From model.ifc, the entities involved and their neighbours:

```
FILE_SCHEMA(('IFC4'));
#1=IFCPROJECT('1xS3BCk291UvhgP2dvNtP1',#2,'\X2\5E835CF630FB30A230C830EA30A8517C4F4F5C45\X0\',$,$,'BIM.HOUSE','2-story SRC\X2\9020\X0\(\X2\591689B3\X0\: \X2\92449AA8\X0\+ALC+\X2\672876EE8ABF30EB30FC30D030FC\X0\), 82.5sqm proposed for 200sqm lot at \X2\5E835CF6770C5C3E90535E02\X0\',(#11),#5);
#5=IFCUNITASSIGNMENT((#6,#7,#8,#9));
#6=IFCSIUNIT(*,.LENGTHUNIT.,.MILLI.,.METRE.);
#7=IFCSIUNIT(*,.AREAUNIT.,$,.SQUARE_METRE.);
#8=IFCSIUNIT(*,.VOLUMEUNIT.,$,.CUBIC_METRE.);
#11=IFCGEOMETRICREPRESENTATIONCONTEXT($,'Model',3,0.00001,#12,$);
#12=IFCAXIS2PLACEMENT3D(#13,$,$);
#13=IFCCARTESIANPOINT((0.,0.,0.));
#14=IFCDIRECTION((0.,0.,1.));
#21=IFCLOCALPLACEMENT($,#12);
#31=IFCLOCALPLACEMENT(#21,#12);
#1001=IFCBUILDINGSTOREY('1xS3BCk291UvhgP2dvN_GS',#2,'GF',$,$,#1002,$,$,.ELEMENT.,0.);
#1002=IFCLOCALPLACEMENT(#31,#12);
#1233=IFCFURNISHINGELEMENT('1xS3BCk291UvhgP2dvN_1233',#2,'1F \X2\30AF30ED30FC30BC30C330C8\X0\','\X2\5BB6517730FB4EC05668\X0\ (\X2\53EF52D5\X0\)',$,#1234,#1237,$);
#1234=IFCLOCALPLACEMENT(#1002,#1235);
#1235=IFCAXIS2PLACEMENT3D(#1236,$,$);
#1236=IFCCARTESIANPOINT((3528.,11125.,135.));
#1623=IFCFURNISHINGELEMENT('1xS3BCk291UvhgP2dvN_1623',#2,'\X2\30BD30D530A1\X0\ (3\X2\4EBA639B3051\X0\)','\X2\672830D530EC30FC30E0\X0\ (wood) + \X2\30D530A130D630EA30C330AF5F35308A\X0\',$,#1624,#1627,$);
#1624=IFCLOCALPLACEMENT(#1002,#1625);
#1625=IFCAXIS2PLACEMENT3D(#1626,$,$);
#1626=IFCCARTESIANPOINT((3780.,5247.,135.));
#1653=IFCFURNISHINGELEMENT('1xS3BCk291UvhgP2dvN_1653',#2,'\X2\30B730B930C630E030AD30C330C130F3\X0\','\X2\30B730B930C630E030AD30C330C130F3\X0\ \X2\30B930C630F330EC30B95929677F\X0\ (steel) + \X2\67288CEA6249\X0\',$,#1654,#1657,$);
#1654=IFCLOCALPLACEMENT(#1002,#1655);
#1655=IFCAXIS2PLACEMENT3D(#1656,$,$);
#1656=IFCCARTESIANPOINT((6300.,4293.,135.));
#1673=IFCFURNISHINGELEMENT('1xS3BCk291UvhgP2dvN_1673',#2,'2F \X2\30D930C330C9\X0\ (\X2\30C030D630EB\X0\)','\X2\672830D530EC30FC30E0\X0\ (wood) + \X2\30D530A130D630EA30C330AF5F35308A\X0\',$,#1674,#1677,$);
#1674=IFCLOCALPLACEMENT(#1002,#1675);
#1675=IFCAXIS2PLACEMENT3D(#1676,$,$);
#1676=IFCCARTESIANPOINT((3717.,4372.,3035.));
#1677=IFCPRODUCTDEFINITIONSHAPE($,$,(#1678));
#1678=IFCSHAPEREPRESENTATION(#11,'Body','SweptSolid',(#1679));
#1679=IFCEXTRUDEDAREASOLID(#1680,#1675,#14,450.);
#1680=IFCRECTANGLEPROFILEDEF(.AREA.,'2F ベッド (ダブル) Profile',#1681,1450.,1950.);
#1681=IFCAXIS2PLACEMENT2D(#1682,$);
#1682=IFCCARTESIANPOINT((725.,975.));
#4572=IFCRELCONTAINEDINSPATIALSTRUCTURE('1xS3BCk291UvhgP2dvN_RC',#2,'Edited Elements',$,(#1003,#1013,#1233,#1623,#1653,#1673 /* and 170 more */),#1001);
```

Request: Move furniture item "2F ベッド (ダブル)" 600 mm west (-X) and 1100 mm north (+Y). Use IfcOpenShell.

```python
import ifcopenshell
import ifcopenshell.api.geometry
import ifcopenshell.util.placement

model = ifcopenshell.open("model.ifc")

item = model.by_id(1673)
matrix = ifcopenshell.util.placement.get_local_placement(item.ObjectPlacement)
matrix[0, 3] -= 600.0
matrix[1, 3] += 1100.0
ifcopenshell.api.geometry.edit_object_placement(model, product=item, matrix=matrix, is_si=False)

print(ifcopenshell.util.placement.get_local_placement(item.ObjectPlacement).round(3) + 0.0)

model.write("model_edited.ifc")
```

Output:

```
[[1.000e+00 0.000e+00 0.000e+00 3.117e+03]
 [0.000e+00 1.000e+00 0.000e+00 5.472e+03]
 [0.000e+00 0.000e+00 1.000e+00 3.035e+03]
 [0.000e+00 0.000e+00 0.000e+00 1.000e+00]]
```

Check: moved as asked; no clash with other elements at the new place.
